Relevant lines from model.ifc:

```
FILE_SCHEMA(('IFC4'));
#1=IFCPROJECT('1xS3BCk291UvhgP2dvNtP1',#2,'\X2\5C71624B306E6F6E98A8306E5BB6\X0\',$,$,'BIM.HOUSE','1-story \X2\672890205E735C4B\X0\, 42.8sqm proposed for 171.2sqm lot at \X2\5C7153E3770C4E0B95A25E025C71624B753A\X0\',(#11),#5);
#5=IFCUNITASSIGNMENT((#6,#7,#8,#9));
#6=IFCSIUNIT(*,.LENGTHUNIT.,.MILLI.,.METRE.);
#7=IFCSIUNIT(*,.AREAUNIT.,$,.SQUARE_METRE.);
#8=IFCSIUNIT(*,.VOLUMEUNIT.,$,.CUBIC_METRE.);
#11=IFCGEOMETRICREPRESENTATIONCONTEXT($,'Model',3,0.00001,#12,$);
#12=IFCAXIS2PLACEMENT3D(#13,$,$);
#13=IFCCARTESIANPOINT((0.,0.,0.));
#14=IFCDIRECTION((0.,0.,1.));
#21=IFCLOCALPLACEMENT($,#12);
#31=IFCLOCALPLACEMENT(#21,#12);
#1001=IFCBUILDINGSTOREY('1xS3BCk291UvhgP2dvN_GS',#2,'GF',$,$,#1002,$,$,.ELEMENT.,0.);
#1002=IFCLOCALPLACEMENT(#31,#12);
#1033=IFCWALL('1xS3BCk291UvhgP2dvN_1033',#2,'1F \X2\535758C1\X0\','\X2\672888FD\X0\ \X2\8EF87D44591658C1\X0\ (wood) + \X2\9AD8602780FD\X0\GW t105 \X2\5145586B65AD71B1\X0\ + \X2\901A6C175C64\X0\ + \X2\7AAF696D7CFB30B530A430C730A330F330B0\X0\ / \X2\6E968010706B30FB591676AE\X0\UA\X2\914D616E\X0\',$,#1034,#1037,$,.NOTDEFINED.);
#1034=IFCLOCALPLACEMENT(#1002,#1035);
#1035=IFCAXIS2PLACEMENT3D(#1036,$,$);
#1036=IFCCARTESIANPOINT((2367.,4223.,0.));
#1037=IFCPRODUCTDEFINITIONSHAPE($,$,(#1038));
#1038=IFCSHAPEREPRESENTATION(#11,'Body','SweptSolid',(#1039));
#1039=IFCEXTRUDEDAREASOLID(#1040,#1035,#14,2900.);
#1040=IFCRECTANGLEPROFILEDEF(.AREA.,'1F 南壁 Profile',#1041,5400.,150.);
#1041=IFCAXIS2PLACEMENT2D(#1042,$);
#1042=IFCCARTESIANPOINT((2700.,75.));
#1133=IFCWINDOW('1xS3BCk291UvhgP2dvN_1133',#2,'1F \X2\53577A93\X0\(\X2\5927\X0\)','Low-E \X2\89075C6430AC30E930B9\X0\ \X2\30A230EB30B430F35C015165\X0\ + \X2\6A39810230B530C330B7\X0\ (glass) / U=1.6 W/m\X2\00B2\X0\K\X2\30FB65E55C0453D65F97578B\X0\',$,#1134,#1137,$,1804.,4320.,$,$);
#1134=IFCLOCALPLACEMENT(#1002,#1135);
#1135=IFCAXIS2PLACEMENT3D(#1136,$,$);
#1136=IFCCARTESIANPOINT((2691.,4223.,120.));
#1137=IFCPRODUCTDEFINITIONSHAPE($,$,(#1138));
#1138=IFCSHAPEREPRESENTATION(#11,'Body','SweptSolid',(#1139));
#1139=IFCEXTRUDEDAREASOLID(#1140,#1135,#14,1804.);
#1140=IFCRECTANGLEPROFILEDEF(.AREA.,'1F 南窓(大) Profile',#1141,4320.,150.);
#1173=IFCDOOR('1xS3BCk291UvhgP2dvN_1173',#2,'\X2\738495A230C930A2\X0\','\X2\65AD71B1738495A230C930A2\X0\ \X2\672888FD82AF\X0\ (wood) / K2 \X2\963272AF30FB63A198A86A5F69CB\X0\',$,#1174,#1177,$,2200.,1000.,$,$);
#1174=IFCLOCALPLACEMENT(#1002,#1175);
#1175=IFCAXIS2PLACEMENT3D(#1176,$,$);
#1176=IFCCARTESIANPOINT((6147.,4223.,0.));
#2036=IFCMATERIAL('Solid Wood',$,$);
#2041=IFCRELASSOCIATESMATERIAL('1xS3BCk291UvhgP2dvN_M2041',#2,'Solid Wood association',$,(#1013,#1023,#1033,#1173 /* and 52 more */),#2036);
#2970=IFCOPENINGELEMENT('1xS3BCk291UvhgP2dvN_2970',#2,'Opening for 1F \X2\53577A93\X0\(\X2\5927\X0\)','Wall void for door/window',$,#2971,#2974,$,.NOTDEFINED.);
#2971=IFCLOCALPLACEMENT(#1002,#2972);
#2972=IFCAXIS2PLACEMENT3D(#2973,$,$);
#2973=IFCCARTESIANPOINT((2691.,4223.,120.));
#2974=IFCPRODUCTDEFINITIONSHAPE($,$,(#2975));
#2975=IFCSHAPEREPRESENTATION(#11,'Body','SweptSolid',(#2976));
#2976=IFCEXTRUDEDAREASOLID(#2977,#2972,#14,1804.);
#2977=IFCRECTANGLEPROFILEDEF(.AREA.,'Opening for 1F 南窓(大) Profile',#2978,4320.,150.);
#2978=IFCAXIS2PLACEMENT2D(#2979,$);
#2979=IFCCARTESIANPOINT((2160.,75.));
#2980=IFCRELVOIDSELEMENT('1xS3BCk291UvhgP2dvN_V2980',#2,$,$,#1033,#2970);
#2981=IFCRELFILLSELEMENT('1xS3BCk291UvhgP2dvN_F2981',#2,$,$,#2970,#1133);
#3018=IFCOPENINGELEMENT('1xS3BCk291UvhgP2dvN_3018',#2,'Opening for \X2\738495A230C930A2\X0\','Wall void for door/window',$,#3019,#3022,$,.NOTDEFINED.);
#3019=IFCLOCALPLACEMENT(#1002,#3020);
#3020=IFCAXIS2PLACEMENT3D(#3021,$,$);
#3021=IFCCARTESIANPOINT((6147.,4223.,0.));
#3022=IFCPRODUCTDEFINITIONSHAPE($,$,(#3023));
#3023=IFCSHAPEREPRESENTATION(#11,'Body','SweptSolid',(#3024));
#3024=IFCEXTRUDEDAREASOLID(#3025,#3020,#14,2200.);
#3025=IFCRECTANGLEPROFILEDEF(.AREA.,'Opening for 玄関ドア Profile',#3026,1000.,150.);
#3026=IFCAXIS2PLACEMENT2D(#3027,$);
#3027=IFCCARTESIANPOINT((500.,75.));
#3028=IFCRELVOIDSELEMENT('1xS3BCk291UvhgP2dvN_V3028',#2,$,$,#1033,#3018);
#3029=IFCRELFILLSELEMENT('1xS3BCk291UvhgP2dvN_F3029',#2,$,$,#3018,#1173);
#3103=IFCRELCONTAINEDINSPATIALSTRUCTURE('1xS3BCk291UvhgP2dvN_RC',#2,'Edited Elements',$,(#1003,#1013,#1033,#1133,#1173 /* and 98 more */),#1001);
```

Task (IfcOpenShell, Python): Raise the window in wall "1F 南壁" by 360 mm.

```python
import numpy as np
import ifcopenshell
import ifcopenshell.api.geometry
import ifcopenshell.util.placement
import ifcopenshell.util.unit

model = ifcopenshell.open("model.ifc")
unit_scale = ifcopenshell.util.unit.calculate_unit_scale(model)

window = model.by_guid("1xS3BCk291UvhgP2dvN_1133")
opening = window.FillsVoids[0].RelatingOpeningElement
dz = 360.0

shift = np.array([0.0, 0.0, dz])
# The window is not placed relative to its opening, so move both.
for product in (opening, window):
    matrix = ifcopenshell.util.placement.get_local_placement(product.ObjectPlacement)
    matrix[:3, 3] += shift
    ifcopenshell.api.geometry.edit_object_placement(model, product=product, matrix=matrix, is_si=False)

print(f"moved by {dz * unit_scale:+.3f} m")

model.write("model_updated.ifc")
```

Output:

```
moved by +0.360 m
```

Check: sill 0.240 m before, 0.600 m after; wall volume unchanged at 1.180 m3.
